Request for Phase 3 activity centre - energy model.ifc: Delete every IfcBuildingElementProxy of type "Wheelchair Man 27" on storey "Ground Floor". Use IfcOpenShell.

First a look at what the model holds.

```python
import ifcopenshell
import ifcopenshell.util.element

model = ifcopenshell.open("Phase 3 activity centre - energy model.ifc")
print(model.schema)
storey = next(s for s in model.by_type("IfcBuildingStorey") if s.Name == "Ground Floor")
proxies = [e for e in ifcopenshell.util.element.get_decomposition(storey) if e.is_a("IfcBuildingElementProxy")]
seen = {}
for e in proxies:
    element_type = ifcopenshell.util.element.get_type(e)
    name = element_type.Name if element_type not in (None, e) else None
    seen[name] = seen.get(name, 0) + 1
for name, count in sorted(seen.items(), key=str):
    print(count, "x", name)
```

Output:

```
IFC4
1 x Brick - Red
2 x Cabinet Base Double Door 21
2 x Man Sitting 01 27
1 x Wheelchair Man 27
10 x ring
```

```python
import ifcopenshell
import ifcopenshell.api.root
import ifcopenshell.util.element

model = ifcopenshell.open("Phase 3 activity centre - energy model.ifc")

storey = next(s for s in model.by_type("IfcBuildingStorey") if s.Name == "Ground Floor")
proxies = [e for e in ifcopenshell.util.element.get_decomposition(storey) if e.is_a("IfcBuildingElementProxy")]
targets = [e for e in proxies if (t := ifcopenshell.util.element.get_type(e)) not in (None, e) and t.Name == "Wheelchair Man 27"]

for e in targets:
    ifcopenshell.api.root.remove_product(model, product=e)
print(len(targets), "removed")

model.write("Phase 3 activity centre - energy model-out.ifc")
```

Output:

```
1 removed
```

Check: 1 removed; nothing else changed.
